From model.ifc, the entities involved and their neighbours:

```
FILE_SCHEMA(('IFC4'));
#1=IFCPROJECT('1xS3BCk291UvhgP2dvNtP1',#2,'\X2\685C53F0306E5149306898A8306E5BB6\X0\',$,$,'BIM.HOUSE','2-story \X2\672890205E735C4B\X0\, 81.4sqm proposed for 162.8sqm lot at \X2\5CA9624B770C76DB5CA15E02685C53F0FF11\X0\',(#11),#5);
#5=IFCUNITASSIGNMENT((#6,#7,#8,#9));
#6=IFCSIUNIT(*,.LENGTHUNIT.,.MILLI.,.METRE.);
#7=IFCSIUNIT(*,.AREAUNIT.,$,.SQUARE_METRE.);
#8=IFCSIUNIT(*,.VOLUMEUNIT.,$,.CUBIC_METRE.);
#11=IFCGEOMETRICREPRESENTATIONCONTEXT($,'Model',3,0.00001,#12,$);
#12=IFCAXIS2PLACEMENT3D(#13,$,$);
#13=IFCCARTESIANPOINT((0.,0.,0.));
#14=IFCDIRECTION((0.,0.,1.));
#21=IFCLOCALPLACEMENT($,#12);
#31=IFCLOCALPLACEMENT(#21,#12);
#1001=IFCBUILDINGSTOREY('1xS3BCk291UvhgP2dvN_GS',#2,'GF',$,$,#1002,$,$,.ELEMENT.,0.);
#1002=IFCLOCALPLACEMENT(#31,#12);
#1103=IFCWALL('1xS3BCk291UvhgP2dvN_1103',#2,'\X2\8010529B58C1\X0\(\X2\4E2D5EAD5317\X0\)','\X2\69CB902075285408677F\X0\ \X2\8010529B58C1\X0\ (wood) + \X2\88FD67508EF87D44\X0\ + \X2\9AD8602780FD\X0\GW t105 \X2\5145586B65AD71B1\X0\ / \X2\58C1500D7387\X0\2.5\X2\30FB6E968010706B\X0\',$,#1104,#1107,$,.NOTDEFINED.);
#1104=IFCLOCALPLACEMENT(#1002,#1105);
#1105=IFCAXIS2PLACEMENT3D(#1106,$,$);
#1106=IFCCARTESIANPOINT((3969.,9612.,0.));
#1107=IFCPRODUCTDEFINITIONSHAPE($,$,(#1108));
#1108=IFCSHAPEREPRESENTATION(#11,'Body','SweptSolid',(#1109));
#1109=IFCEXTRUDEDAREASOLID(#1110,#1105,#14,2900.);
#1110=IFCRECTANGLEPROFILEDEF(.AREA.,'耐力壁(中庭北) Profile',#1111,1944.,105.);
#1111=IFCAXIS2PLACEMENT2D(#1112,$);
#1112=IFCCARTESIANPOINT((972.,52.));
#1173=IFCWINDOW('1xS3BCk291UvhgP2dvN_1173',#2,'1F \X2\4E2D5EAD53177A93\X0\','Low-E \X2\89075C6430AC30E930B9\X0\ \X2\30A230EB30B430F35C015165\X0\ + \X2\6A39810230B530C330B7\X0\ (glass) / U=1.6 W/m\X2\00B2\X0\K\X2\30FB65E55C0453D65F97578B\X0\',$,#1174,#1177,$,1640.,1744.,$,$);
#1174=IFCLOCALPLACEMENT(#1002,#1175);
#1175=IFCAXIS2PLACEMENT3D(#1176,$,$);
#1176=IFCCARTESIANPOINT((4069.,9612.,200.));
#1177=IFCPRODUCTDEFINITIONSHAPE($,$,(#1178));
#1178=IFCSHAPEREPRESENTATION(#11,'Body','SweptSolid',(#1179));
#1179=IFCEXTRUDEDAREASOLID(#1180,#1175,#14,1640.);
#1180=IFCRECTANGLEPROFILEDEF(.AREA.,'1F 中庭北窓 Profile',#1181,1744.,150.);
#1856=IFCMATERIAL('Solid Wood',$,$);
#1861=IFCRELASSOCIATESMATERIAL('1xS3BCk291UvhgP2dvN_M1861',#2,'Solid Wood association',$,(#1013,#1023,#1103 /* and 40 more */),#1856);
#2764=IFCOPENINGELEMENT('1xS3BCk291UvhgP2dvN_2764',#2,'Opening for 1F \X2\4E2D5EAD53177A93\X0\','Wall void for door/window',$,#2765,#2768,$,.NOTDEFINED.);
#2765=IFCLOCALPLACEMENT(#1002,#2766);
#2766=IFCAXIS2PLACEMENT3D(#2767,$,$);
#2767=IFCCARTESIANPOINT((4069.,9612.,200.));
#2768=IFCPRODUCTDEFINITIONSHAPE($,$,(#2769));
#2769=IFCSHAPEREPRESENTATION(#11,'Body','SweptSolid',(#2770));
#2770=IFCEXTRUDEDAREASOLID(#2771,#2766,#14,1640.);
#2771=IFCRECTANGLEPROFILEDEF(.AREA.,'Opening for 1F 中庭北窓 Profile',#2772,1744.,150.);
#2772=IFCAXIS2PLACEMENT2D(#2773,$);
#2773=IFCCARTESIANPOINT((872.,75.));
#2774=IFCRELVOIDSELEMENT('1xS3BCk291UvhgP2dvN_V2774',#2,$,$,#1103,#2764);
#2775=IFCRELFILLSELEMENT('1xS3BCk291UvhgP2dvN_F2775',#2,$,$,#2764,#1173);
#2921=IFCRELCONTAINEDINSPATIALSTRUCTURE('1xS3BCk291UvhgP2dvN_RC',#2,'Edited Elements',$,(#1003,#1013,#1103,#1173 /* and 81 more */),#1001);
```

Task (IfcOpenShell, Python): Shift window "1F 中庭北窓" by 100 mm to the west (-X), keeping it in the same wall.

```python
import ifcopenshell
import ifcopenshell.api.geometry
import ifcopenshell.util.placement
import ifcopenshell.util.unit

model = ifcopenshell.open("model.ifc")
unit_scale = ifcopenshell.util.unit.calculate_unit_scale(model)

window = model.by_id(1173)
opening = window.FillsVoids[0].RelatingOpeningElement
wall = opening.VoidsElements[0].RelatingBuildingElement

wall_matrix = ifcopenshell.util.placement.get_local_placement(wall.ObjectPlacement)
shift = wall_matrix[:3, 0] * -0.1 / unit_scale
before = ifcopenshell.util.placement.get_local_placement(window.ObjectPlacement)[:3, 3].copy()

# The window is not placed relative to its opening, so move both.
for product in (opening, window):
    matrix = ifcopenshell.util.placement.get_local_placement(product.ObjectPlacement)
    matrix[:3, 3] += shift
    ifcopenshell.api.geometry.edit_object_placement(model, product=product, matrix=matrix, is_si=False)

after = ifcopenshell.util.placement.get_local_placement(window.ObjectPlacement)[:3, 3]
print("window moved by", (after - before).round(3) + 0.0)

model.write("model_edited.ifc")
```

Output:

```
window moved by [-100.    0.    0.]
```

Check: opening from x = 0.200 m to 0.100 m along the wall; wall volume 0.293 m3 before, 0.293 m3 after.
